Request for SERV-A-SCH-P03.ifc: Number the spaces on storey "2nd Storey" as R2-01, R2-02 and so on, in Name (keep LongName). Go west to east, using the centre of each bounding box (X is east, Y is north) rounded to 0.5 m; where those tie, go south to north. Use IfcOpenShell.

First a look at what the model holds.

```python
import ifcopenshell
import ifcopenshell.util.element
import ifcopenshell.util.placement

model = ifcopenshell.open("SERV-A-SCH-P03.ifc")
print(model.schema)
storey = next(s for s in model.by_type("IfcBuildingStorey") if s.Name == "2nd Storey")
spaces = [e for e in ifcopenshell.util.element.get_decomposition(storey) if e.is_a("IfcSpace")]
for e in sorted(spaces, key=lambda e: e.id()):
    origin = ifcopenshell.util.placement.get_local_placement(e.ObjectPlacement)[:3, 3]
    print(e.id(), e.Name, e.LongName, origin.round(2) + 0.0, sep=" | ")
```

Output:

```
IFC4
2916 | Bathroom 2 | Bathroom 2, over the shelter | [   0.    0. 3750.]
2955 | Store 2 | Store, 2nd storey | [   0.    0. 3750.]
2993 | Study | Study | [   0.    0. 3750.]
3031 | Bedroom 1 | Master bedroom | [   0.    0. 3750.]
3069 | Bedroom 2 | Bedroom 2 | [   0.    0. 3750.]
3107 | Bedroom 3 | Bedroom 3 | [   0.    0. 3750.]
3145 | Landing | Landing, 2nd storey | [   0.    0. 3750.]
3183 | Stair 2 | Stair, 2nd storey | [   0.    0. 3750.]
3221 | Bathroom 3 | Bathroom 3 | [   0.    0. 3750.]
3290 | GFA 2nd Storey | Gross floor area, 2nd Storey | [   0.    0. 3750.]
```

```python
import ifcopenshell
import ifcopenshell.geom
import ifcopenshell.util.element
import ifcopenshell.util.shape

model = ifcopenshell.open("SERV-A-SCH-P03.ifc")
settings = ifcopenshell.geom.settings()
settings.set("use-world-coords", True)


def centre(element):
    shape = ifcopenshell.geom.create_shape(settings, element)
    return ifcopenshell.util.shape.get_bbox_centroid(shape.geometry)


storey = next(s for s in model.by_type("IfcBuildingStorey") if s.Name == "2nd Storey")
spaces = [e for e in ifcopenshell.util.element.get_decomposition(storey) if e.is_a("IfcSpace")]

# Insertion points can sit at a corner or the storey origin, so sort by the geometry (in metres).
centres = {e: centre(e) for e in spaces}
spaces.sort(key=lambda e: (round(centres[e][0] / 0.5), centres[e][1]))

for i, e in enumerate(spaces, start=1):
    number = f"R2-{i:02d}"
    e.Name = number
    print(e.id(), number)

model.write("SERV-A-SCH-P03_rev.ifc")
```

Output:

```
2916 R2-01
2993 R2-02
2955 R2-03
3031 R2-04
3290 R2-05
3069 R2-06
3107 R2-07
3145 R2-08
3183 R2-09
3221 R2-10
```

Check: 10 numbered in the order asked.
